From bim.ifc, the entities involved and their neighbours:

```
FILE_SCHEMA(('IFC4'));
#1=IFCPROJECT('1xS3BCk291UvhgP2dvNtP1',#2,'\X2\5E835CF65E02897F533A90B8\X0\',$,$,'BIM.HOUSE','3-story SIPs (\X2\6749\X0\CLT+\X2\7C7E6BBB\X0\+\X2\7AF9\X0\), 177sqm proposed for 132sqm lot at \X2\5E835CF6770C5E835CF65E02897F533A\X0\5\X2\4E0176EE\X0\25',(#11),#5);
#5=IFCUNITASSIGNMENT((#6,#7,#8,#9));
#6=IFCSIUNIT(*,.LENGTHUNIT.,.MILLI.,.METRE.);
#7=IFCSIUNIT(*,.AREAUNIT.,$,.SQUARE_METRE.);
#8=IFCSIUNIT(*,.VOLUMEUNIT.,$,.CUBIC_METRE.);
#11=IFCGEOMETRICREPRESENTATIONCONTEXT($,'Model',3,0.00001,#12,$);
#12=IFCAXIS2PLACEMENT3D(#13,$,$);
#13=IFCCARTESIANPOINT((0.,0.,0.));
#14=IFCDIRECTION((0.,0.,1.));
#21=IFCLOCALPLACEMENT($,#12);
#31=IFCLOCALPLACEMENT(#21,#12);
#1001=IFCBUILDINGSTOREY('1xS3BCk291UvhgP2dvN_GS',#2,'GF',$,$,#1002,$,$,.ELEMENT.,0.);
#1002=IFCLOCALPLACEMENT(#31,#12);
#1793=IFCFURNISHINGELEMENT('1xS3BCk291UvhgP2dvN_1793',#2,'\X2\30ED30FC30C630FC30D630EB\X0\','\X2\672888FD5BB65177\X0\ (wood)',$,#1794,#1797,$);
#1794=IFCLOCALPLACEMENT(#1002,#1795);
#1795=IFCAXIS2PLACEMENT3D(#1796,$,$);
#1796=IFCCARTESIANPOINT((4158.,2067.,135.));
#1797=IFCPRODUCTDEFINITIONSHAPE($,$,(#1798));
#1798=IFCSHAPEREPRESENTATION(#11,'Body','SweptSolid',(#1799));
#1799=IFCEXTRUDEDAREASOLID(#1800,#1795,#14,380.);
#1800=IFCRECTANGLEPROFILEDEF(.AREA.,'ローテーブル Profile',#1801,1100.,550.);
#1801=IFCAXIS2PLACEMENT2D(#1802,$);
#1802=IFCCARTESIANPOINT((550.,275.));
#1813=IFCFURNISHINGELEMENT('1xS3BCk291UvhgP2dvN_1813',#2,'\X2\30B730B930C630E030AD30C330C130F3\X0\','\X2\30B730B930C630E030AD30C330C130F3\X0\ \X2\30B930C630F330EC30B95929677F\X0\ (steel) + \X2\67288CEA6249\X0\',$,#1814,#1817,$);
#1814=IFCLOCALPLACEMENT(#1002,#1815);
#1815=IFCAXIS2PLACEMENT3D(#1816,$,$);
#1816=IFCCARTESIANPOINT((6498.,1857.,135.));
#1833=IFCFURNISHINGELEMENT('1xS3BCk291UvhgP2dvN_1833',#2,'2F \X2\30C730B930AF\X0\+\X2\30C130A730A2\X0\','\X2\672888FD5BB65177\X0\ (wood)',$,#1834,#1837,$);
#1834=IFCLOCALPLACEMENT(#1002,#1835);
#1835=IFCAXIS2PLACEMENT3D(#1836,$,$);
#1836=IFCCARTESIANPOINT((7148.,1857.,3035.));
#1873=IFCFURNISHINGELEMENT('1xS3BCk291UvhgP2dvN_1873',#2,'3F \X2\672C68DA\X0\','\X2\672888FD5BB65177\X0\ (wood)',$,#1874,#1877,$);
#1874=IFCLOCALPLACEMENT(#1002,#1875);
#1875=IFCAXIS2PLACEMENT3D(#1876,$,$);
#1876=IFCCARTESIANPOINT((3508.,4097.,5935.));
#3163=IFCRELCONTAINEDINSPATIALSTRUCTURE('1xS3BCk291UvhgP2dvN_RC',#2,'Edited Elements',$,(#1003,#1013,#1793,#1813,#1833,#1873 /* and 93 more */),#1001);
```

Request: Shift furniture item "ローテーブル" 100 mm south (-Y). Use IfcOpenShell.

```python
import ifcopenshell
import ifcopenshell.api.geometry
import ifcopenshell.util.placement
import ifcopenshell.util.unit

model = ifcopenshell.open("bim.ifc")
unit_scale = ifcopenshell.util.unit.calculate_unit_scale(model)

item = model.by_guid("1xS3BCk291UvhgP2dvN_1793")
matrix = ifcopenshell.util.placement.get_local_placement(item.ObjectPlacement)
matrix[1, 3] -= 0.1 / unit_scale
ifcopenshell.api.geometry.edit_object_placement(model, product=item, matrix=matrix, is_si=False)

print(ifcopenshell.util.placement.get_local_placement(item.ObjectPlacement).round(3) + 0.0)

model.write("bim_edited.ifc")
```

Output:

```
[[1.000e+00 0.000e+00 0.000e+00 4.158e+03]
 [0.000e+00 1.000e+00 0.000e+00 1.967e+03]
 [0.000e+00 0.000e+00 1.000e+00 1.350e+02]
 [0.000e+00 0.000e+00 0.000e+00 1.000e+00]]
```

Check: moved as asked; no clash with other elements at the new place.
